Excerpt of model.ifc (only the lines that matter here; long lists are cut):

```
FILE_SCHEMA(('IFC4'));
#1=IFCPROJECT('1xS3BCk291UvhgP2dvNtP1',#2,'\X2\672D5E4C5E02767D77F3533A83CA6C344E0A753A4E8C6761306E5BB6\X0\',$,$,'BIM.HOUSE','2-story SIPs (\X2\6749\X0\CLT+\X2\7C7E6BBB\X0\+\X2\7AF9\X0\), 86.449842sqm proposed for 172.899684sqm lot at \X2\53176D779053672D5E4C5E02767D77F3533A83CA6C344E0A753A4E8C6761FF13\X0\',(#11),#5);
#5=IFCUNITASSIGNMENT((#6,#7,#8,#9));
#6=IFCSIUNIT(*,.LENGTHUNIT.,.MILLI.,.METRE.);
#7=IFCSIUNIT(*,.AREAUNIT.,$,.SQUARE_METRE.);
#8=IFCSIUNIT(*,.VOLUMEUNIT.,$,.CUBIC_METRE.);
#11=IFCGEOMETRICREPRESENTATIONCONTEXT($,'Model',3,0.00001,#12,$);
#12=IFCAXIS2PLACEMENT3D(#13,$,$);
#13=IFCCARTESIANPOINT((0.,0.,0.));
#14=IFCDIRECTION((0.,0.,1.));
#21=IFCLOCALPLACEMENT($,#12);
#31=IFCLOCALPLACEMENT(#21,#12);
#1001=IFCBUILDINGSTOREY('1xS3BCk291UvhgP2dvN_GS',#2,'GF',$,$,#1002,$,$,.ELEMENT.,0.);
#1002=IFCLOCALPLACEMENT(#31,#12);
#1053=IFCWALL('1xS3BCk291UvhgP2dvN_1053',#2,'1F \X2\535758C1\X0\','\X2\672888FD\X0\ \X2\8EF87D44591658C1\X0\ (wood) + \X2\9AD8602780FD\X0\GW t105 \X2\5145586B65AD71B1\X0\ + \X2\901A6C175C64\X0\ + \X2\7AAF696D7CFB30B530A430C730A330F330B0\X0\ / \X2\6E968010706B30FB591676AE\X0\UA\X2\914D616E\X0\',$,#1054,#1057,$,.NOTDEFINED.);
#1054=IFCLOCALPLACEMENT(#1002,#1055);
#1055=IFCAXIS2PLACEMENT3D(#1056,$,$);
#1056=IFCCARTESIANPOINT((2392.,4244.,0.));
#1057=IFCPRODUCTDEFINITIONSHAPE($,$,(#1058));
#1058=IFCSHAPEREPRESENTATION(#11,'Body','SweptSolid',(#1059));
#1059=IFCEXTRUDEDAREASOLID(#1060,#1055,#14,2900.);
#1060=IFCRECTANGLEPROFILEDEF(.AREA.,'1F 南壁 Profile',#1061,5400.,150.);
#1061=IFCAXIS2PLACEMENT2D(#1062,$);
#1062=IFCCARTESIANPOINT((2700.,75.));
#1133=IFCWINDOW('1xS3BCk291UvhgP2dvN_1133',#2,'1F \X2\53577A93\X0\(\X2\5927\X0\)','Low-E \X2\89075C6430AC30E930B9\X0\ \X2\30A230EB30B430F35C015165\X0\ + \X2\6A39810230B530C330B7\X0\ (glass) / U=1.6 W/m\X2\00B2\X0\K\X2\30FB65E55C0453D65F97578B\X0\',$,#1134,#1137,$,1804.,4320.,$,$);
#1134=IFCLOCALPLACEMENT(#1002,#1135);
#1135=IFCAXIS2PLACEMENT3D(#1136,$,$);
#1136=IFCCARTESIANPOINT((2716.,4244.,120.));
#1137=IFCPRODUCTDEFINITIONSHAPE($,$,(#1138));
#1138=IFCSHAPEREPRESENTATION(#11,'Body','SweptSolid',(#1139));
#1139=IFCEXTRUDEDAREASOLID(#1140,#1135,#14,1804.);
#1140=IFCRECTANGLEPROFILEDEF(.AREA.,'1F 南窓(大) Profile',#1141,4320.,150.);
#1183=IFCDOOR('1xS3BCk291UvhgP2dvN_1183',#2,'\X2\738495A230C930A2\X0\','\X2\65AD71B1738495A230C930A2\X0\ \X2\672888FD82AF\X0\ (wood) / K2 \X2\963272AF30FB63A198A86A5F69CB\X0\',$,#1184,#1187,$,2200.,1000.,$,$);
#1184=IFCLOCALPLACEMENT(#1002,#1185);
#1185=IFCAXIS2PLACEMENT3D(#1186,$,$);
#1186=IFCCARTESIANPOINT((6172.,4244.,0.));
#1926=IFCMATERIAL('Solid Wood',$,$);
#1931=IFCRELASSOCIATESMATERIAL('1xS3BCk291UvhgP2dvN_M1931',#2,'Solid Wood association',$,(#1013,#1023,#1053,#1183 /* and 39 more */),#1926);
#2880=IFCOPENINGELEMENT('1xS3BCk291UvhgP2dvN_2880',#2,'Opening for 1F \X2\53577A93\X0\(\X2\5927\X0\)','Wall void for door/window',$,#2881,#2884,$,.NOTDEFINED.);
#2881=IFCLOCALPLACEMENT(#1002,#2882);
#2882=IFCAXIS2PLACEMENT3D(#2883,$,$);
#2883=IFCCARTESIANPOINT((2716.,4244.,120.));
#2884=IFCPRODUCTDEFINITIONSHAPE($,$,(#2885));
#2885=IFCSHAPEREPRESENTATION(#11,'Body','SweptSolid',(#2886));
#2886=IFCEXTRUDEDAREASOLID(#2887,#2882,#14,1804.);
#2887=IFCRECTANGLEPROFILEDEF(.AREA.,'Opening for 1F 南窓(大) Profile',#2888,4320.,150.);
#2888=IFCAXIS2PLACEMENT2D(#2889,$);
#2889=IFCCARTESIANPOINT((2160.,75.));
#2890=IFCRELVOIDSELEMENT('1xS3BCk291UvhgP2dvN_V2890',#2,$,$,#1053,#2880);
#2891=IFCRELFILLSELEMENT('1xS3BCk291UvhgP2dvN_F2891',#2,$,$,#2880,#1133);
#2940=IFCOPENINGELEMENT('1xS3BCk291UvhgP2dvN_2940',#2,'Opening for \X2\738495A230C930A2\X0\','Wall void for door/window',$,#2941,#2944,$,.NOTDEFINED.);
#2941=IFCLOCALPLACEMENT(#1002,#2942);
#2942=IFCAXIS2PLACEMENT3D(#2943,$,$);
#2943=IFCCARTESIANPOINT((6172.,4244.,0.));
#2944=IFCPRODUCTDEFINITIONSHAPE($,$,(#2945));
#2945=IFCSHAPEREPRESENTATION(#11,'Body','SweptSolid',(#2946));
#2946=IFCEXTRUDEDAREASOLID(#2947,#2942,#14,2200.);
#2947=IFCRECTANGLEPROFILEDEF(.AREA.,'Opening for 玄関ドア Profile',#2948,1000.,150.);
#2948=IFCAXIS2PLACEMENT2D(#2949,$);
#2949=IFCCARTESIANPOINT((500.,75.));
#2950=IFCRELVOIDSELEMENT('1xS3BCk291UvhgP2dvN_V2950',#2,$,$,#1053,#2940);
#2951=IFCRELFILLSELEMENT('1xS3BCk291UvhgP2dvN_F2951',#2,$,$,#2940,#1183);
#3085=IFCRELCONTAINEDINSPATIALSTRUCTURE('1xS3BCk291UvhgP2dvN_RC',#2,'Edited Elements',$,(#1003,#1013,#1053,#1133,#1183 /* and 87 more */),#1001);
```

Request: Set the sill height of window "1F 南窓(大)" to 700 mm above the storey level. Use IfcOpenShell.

```python
import numpy as np
import ifcopenshell
import ifcopenshell.api.geometry
import ifcopenshell.geom
import ifcopenshell.util.element
import ifcopenshell.util.placement
import ifcopenshell.util.shape
import ifcopenshell.util.unit

model = ifcopenshell.open("model.ifc")
unit_scale = ifcopenshell.util.unit.calculate_unit_scale(model)

window = model.by_guid("1xS3BCk291UvhgP2dvN_1133")
opening = window.FillsVoids[0].RelatingOpeningElement
storey = ifcopenshell.util.element.get_container(window, ifc_class="IfcBuildingStorey")
level = ifcopenshell.util.placement.get_local_placement(storey.ObjectPlacement)[2, 3]

# The opening's origin need not be at the sill, so measure its lowest point.
shape = ifcopenshell.geom.create_shape(ifcopenshell.geom.settings(), opening)
bottom = ifcopenshell.util.shape.get_shape_bottom_elevation(shape, shape.geometry) / unit_scale
dz = level + 0.7 / unit_scale - bottom

shift = np.array([0.0, 0.0, dz])
# The window is not placed relative to its opening, so move both.
for product in (opening, window):
    matrix = ifcopenshell.util.placement.get_local_placement(product.ObjectPlacement)
    matrix[:3, 3] += shift
    ifcopenshell.api.geometry.edit_object_placement(model, product=product, matrix=matrix, is_si=False)

print(f"moved by {dz * unit_scale:+.3f} m")

model.write("model_rev.ifc")
```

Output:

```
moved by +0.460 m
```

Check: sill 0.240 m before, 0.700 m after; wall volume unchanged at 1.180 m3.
